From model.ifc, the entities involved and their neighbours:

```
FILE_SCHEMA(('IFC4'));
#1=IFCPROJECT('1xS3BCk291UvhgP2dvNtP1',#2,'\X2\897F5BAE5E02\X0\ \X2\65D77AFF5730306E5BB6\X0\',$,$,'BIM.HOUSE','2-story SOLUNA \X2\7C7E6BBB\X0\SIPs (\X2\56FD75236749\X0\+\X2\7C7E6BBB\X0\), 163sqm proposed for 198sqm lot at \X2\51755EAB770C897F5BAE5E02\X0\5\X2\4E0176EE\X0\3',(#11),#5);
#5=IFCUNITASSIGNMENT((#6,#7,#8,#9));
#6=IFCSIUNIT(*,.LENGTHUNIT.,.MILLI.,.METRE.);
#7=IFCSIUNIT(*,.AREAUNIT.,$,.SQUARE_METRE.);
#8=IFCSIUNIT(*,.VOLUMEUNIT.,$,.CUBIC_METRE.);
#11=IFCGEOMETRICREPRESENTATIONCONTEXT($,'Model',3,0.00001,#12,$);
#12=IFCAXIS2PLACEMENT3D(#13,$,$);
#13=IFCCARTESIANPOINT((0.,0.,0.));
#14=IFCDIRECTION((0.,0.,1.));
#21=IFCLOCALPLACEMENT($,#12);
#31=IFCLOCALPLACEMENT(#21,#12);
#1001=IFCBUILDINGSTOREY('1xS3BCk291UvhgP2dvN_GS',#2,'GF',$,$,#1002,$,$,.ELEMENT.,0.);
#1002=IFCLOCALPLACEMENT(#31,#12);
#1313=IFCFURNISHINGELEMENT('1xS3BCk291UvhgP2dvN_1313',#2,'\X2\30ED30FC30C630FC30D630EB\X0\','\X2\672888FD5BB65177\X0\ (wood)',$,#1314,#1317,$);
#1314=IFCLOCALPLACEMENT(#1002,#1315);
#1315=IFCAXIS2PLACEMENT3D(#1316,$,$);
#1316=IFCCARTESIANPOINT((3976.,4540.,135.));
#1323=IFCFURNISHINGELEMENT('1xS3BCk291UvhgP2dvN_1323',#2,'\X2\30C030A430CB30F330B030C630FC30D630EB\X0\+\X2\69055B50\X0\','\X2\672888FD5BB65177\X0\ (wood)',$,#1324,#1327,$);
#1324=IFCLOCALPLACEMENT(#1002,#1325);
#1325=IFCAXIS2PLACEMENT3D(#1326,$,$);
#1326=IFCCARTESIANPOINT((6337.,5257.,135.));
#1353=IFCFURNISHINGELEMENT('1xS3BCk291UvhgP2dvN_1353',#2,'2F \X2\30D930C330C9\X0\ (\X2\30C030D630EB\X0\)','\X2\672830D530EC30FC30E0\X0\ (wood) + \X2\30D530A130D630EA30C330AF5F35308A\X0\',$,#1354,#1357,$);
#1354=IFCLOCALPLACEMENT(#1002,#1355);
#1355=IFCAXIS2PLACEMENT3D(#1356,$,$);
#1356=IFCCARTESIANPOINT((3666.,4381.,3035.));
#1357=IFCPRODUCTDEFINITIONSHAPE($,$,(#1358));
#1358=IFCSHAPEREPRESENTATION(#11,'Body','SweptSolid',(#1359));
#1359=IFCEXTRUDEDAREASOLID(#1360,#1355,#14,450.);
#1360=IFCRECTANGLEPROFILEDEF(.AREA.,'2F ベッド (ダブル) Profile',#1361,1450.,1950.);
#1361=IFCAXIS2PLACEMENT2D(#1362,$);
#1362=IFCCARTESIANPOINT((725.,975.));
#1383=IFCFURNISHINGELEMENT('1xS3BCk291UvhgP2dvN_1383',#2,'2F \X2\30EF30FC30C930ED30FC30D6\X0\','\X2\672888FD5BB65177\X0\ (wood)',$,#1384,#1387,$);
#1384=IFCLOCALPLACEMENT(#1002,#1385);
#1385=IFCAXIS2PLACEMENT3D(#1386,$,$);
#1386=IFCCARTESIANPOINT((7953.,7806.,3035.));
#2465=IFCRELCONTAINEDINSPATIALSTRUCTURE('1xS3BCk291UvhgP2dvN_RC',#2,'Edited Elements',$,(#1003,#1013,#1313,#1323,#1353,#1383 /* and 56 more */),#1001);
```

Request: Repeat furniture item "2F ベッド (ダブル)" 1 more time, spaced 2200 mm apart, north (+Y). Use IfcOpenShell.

```python
import numpy as np
import ifcopenshell
import ifcopenshell.api.geometry
import ifcopenshell.api.root
import ifcopenshell.util.element
import ifcopenshell.util.placement
import ifcopenshell.util.unit

model = ifcopenshell.open("model.ifc")
unit_scale = ifcopenshell.util.unit.calculate_unit_scale(model)


def reuse_history(source, copy):
    """copy_class also copies each property set's owner history, people and application; keep the originals."""
    for rel in copy.IsDefinedBy:
        if rel.is_a("IfcRelDefinesByProperties") and (history := rel.RelatingPropertyDefinition.OwnerHistory):
            rel.RelatingPropertyDefinition.OwnerHistory = source.OwnerHistory
            ifcopenshell.util.element.remove_deep2(model, history)


source = model.by_guid("1xS3BCk291UvhgP2dvN_1353")
base = ifcopenshell.util.placement.get_local_placement(source.ObjectPlacement)
step = np.array([0.0, 1.0, 0.0]) * 2.2 / unit_scale

for i in range(1, 2):
    copy = ifcopenshell.api.root.copy_class(model, product=source)
    copy.Representation = ifcopenshell.util.element.copy_deep(
        model, source.Representation, exclude=["IfcGeometricRepresentationContext", "IfcRepresentationMap"]
    )
    reuse_history(source, copy)
    matrix = base.copy()
    matrix[:3, 3] += i * step
    print("added at", matrix[:3, 3].round(3) + 0.0)
    ifcopenshell.api.geometry.edit_object_placement(model, product=copy, matrix=matrix, is_si=False)

model.write("model_edited.ifc")
```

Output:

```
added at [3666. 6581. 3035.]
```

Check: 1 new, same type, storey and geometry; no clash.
